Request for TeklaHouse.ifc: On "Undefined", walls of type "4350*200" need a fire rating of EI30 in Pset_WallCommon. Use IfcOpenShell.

First a look at what the model holds.

```python
import ifcopenshell
import ifcopenshell.util.element

model = ifcopenshell.open("TeklaHouse.ifc")
print(model.schema)
storey = next(s for s in model.by_type("IfcBuildingStorey") if s.Name == "Undefined")
walls = [e for e in ifcopenshell.util.element.get_decomposition(storey) if e.is_a("IfcWall")]
seen = {}
for e in walls:
    element_type = ifcopenshell.util.element.get_type(e)
    key = (element_type.Name if element_type != e and element_type else None, ifcopenshell.util.element.get_pset(e, "Pset_WallCommon", "FireRating"))
    seen[key] = seen.get(key, 0) + 1
for (name, value), count in sorted(seen.items(), key=str):
    print(count, "x", name, "|", value)
```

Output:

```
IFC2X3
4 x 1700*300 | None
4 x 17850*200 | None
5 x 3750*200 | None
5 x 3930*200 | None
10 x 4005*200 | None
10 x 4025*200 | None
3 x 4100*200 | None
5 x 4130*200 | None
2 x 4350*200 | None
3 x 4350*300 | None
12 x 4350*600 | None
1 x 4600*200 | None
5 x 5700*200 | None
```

```python
import ifcopenshell
import ifcopenshell.api.pset
import ifcopenshell.util.element

model = ifcopenshell.open("TeklaHouse.ifc")

storey = next(s for s in model.by_type("IfcBuildingStorey") if s.Name == "Undefined")
walls = [e for e in ifcopenshell.util.element.get_decomposition(storey) if e.is_a("IfcWall")]

count = 0
for e in walls:
    element_type = ifcopenshell.util.element.get_type(e)
    if element_type in (None, e) or element_type.Name != "4350*200":
        continue
    # add_pset returns the element's existing set when there is one.
    pset = ifcopenshell.api.pset.add_pset(model, product=e, name="Pset_WallCommon")
    ifcopenshell.api.pset.edit_pset(model, pset=pset, properties={"FireRating": "EI30"})
    count += 1

print(count, "walls updated")

model.write("TeklaHouse_rev.ifc")
```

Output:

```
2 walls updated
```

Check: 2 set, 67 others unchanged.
